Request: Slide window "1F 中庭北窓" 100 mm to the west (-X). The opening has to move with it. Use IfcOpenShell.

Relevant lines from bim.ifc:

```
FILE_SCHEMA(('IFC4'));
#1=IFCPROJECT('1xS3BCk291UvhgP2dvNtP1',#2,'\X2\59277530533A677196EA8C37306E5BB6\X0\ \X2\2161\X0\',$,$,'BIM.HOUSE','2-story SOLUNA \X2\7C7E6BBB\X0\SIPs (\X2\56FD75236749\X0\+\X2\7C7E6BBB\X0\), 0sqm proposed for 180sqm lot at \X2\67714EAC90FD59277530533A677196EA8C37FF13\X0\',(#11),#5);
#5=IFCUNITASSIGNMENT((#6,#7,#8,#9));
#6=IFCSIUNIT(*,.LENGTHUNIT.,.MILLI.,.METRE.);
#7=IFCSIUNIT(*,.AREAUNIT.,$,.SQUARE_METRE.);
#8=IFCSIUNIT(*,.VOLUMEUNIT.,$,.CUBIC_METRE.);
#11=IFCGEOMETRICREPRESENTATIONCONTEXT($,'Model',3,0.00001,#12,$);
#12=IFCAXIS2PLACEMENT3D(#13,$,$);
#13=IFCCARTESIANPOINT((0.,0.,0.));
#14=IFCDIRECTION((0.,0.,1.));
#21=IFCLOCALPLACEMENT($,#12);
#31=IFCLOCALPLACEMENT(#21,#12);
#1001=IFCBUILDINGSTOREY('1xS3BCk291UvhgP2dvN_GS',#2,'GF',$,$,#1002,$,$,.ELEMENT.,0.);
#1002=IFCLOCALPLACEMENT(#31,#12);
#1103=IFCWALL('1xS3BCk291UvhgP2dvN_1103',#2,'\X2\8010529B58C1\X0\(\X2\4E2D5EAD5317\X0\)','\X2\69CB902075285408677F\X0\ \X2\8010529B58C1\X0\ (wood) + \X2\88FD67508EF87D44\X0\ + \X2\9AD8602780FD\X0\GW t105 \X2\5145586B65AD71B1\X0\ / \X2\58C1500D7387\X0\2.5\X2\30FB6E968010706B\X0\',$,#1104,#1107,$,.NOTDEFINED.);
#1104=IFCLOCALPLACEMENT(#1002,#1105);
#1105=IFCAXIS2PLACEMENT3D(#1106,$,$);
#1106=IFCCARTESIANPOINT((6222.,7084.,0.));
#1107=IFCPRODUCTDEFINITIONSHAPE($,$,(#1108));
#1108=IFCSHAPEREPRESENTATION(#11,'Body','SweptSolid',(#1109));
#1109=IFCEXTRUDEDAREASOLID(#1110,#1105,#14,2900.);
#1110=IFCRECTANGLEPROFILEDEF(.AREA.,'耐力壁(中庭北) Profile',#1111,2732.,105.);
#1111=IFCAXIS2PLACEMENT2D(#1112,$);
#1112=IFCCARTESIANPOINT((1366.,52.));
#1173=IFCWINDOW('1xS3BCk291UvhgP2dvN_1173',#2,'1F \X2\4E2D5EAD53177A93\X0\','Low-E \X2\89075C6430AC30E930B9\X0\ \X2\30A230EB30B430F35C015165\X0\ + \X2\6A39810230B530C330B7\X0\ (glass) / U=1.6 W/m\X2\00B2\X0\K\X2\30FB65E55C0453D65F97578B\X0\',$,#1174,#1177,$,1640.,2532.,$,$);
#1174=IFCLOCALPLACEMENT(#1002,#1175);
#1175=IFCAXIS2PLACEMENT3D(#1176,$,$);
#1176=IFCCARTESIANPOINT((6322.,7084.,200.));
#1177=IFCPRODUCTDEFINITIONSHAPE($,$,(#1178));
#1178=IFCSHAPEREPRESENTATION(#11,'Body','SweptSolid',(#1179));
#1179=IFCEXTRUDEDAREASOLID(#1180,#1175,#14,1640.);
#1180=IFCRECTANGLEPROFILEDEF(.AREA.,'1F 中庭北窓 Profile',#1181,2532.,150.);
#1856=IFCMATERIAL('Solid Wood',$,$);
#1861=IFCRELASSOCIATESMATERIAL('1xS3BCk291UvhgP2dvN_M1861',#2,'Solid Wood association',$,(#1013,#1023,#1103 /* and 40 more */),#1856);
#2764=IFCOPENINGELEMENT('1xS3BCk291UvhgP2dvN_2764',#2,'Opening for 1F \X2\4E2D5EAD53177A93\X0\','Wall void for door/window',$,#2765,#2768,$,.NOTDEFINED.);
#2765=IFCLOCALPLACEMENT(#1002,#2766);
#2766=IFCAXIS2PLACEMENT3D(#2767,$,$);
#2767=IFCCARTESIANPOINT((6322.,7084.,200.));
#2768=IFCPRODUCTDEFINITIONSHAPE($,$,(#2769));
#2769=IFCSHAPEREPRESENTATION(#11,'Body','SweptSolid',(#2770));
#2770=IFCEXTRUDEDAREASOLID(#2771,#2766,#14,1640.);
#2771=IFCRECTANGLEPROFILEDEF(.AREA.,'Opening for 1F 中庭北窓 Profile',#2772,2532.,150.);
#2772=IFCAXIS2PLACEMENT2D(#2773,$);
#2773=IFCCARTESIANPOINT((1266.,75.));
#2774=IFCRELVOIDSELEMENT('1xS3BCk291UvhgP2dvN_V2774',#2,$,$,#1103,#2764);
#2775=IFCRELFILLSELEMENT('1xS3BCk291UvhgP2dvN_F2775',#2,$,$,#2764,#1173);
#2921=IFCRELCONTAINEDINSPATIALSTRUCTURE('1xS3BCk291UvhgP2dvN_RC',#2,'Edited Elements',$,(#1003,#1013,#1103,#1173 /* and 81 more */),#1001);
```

```python
import ifcopenshell
import ifcopenshell.api.geometry
import ifcopenshell.util.placement

model = ifcopenshell.open("bim.ifc")

window = model.by_guid("1xS3BCk291UvhgP2dvN_1173")
opening = window.FillsVoids[0].RelatingOpeningElement
wall = opening.VoidsElements[0].RelatingBuildingElement

wall_matrix = ifcopenshell.util.placement.get_local_placement(wall.ObjectPlacement)
shift = wall_matrix[:3, 0] * -100.0
before = ifcopenshell.util.placement.get_local_placement(window.ObjectPlacement)[:3, 3].copy()

# The window is not placed relative to its opening, so move both.
for product in (opening, window):
    matrix = ifcopenshell.util.placement.get_local_placement(product.ObjectPlacement)
    matrix[:3, 3] += shift
    ifcopenshell.api.geometry.edit_object_placement(model, product=product, matrix=matrix, is_si=False)

after = ifcopenshell.util.placement.get_local_placement(window.ObjectPlacement)[:3, 3]
print("window moved by", (after - before).round(3) + 0.0)

model.write("bim_edited.ifc")
```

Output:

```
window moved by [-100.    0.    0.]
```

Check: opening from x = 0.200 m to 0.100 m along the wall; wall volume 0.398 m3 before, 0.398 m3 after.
